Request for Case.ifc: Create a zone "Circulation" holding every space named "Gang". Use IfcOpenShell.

First a look at what the model holds.

```python
import ifcopenshell

model = ifcopenshell.open("Case.ifc")
print(model.schema)
seen = {}
for space in model.by_type("IfcSpace"):
    seen[space.LongName] = seen.get(space.LongName, 0) + 1
for name, count in sorted(seen.items(), key=str):
    print(count, "x", name)
print("zones:", [z.Name for z in model.by_type("IfcZone")][:20])
```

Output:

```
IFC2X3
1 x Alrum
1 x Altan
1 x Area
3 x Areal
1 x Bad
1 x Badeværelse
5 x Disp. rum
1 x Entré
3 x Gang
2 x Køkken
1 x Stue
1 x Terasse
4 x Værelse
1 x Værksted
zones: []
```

```python
import ifcopenshell
import ifcopenshell.api.group
import ifcopenshell.api.root

model = ifcopenshell.open("Case.ifc")

names = {"Gang"}
spaces = [s for s in model.by_type("IfcSpace") if s.LongName in names]

zone = ifcopenshell.api.root.create_entity(model, ifc_class="IfcZone", name="Circulation")
ifcopenshell.api.group.assign_group(model, products=spaces, group=zone)
print(len(spaces), "spaces in", zone.Name)

model.write("Case_edited.ifc")
```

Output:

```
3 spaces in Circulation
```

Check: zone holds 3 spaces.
